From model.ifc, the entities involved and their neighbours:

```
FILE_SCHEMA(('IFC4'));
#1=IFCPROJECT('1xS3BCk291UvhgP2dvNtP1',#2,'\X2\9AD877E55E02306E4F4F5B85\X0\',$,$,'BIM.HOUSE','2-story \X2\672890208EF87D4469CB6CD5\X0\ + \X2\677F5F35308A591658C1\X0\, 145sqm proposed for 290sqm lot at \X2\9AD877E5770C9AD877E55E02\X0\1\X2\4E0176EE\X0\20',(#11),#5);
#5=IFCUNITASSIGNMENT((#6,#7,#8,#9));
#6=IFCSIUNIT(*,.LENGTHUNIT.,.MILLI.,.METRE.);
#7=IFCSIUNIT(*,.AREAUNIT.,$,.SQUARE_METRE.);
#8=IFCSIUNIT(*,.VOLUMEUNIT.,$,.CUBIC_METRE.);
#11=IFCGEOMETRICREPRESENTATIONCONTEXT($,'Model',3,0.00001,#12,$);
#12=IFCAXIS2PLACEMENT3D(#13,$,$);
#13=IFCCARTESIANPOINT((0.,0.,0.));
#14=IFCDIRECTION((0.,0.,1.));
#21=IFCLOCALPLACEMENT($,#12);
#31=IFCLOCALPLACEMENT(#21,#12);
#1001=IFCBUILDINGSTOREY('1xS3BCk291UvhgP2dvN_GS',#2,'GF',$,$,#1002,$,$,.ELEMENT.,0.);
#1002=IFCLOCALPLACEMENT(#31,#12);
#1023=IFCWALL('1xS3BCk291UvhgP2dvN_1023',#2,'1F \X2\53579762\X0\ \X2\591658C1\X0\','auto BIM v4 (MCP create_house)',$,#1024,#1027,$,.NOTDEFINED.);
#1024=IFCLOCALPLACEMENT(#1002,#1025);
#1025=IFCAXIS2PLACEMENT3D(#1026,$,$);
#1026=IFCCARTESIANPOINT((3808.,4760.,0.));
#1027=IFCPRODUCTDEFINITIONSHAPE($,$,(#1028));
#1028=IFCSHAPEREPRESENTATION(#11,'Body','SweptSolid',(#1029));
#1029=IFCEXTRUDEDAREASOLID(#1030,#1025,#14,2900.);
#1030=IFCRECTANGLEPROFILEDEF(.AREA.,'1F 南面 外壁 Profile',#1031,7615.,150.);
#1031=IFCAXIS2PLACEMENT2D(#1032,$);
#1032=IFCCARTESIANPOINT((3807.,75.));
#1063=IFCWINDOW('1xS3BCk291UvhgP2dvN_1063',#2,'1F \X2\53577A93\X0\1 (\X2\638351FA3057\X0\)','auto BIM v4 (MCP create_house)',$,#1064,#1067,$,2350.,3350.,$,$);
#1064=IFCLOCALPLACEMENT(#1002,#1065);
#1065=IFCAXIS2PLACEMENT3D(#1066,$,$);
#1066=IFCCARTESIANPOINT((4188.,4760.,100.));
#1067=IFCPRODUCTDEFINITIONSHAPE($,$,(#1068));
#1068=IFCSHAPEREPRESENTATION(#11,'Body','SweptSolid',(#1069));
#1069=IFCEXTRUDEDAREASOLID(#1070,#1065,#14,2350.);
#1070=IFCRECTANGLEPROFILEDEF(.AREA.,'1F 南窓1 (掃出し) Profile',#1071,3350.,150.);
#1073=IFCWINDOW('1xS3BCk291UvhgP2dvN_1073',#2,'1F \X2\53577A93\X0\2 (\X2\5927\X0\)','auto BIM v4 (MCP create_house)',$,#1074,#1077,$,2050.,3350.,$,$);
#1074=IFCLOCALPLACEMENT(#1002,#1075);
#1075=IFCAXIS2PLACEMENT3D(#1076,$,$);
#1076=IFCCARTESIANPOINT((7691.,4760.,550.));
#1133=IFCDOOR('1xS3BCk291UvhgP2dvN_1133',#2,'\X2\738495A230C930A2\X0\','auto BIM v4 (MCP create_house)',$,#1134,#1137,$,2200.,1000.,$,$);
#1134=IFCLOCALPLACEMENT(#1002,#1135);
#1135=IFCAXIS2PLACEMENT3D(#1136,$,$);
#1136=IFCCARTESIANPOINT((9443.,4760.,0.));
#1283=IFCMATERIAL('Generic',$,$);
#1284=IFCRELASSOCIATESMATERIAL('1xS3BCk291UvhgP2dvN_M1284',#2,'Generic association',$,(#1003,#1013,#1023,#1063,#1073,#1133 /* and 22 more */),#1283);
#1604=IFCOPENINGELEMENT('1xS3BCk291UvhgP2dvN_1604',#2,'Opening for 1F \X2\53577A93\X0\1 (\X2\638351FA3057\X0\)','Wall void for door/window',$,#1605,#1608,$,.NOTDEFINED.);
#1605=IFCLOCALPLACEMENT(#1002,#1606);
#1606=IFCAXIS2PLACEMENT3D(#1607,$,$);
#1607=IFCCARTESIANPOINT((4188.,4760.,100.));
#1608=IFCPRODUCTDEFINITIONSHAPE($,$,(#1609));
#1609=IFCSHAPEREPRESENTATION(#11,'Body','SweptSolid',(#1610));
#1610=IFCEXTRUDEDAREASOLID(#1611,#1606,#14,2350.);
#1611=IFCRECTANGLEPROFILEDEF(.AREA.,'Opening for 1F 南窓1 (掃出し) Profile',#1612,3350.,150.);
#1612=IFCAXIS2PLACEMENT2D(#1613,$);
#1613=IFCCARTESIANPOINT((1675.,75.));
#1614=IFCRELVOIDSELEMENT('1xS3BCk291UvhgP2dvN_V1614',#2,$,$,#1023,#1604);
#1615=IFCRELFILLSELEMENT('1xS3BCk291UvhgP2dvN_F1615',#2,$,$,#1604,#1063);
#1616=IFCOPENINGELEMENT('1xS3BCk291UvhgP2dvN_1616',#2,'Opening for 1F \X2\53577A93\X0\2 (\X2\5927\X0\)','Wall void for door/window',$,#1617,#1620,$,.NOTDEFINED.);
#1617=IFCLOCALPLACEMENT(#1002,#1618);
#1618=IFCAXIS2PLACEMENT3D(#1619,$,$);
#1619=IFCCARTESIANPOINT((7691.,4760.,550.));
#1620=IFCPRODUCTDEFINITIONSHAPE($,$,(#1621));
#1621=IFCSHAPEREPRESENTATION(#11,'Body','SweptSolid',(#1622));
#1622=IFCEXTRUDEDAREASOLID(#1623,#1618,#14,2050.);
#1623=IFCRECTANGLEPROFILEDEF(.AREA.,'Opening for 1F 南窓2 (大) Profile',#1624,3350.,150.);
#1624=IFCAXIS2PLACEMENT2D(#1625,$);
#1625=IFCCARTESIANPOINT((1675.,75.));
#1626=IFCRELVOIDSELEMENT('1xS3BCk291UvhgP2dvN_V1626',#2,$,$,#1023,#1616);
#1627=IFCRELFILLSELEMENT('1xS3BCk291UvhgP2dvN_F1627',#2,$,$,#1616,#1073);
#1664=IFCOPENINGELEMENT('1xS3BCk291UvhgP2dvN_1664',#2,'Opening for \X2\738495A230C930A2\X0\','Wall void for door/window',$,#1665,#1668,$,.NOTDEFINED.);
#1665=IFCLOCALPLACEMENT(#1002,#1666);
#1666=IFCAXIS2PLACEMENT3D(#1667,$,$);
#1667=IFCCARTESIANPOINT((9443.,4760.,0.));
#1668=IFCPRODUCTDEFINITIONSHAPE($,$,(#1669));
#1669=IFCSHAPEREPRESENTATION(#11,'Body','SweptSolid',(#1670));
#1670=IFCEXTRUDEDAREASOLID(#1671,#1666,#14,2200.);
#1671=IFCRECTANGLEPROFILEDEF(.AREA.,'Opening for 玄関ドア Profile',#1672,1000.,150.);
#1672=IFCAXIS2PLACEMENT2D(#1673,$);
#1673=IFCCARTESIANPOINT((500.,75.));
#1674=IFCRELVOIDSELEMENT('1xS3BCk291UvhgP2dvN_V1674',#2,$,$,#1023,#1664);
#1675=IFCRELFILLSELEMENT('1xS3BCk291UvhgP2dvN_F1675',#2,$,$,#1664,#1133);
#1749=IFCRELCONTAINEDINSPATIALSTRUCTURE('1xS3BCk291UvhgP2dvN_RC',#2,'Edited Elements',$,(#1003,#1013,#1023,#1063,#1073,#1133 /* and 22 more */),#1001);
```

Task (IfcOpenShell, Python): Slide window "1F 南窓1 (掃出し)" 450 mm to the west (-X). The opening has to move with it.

```python
import ifcopenshell
import ifcopenshell.api.geometry
import ifcopenshell.util.placement
import ifcopenshell.util.unit

model = ifcopenshell.open("model.ifc")
unit_scale = ifcopenshell.util.unit.calculate_unit_scale(model)

window = model.by_guid("1xS3BCk291UvhgP2dvN_1063")
opening = window.FillsVoids[0].RelatingOpeningElement
wall = opening.VoidsElements[0].RelatingBuildingElement

wall_matrix = ifcopenshell.util.placement.get_local_placement(wall.ObjectPlacement)
shift = wall_matrix[:3, 0] * -0.45 / unit_scale
before = ifcopenshell.util.placement.get_local_placement(window.ObjectPlacement)[:3, 3].copy()

# The window is not placed relative to its opening, so move both.
for product in (opening, window):
    matrix = ifcopenshell.util.placement.get_local_placement(product.ObjectPlacement)
    matrix[:3, 3] += shift
    ifcopenshell.api.geometry.edit_object_placement(model, product=product, matrix=matrix, is_si=False)

after = ifcopenshell.util.placement.get_local_placement(window.ObjectPlacement)[:3, 3]
print("window moved by", (after - before).round(3) + 0.0)

model.write("model-out.ifc")
```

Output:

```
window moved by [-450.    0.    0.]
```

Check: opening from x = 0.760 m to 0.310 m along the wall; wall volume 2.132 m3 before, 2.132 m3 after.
